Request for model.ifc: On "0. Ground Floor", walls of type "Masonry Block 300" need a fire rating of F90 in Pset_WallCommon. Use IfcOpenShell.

First a look at what the model holds.

```python
import ifcopenshell
import ifcopenshell.util.element

model = ifcopenshell.open("model.ifc")
print(model.schema)
storey = next(s for s in model.by_type("IfcBuildingStorey") if s.Name == "0. Ground Floor")
walls = [e for e in ifcopenshell.util.element.get_decomposition(storey) if e.is_a("IfcWall")]
seen = {}
for e in walls:
    element_type = ifcopenshell.util.element.get_type(e)
    key = (element_type.Name if element_type != e and element_type else None, ifcopenshell.util.element.get_pset(e, "Pset_WallCommon", "FireRating"))
    seen[key] = seen.get(key, 0) + 1
for (name, value), count in sorted(seen.items(), key=str):
    print(count, "x", name, "|", value)
```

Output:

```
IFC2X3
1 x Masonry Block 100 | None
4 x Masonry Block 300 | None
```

```python
import ifcopenshell
import ifcopenshell.api.pset
import ifcopenshell.util.element

model = ifcopenshell.open("model.ifc")

storey = next(s for s in model.by_type("IfcBuildingStorey") if s.Name == "0. Ground Floor")
walls = [e for e in ifcopenshell.util.element.get_decomposition(storey) if e.is_a("IfcWall")]

count = 0
for e in walls:
    element_type = ifcopenshell.util.element.get_type(e)
    if element_type in (None, e) or element_type.Name != "Masonry Block 300":
        continue
    # add_pset returns the element's existing set when there is one.
    pset = ifcopenshell.api.pset.add_pset(model, product=e, name="Pset_WallCommon")
    ifcopenshell.api.pset.edit_pset(model, pset=pset, properties={"FireRating": "F90"})
    count += 1

print(count, "walls updated")

model.write("model_v2.ifc")
```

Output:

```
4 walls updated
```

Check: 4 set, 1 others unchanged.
